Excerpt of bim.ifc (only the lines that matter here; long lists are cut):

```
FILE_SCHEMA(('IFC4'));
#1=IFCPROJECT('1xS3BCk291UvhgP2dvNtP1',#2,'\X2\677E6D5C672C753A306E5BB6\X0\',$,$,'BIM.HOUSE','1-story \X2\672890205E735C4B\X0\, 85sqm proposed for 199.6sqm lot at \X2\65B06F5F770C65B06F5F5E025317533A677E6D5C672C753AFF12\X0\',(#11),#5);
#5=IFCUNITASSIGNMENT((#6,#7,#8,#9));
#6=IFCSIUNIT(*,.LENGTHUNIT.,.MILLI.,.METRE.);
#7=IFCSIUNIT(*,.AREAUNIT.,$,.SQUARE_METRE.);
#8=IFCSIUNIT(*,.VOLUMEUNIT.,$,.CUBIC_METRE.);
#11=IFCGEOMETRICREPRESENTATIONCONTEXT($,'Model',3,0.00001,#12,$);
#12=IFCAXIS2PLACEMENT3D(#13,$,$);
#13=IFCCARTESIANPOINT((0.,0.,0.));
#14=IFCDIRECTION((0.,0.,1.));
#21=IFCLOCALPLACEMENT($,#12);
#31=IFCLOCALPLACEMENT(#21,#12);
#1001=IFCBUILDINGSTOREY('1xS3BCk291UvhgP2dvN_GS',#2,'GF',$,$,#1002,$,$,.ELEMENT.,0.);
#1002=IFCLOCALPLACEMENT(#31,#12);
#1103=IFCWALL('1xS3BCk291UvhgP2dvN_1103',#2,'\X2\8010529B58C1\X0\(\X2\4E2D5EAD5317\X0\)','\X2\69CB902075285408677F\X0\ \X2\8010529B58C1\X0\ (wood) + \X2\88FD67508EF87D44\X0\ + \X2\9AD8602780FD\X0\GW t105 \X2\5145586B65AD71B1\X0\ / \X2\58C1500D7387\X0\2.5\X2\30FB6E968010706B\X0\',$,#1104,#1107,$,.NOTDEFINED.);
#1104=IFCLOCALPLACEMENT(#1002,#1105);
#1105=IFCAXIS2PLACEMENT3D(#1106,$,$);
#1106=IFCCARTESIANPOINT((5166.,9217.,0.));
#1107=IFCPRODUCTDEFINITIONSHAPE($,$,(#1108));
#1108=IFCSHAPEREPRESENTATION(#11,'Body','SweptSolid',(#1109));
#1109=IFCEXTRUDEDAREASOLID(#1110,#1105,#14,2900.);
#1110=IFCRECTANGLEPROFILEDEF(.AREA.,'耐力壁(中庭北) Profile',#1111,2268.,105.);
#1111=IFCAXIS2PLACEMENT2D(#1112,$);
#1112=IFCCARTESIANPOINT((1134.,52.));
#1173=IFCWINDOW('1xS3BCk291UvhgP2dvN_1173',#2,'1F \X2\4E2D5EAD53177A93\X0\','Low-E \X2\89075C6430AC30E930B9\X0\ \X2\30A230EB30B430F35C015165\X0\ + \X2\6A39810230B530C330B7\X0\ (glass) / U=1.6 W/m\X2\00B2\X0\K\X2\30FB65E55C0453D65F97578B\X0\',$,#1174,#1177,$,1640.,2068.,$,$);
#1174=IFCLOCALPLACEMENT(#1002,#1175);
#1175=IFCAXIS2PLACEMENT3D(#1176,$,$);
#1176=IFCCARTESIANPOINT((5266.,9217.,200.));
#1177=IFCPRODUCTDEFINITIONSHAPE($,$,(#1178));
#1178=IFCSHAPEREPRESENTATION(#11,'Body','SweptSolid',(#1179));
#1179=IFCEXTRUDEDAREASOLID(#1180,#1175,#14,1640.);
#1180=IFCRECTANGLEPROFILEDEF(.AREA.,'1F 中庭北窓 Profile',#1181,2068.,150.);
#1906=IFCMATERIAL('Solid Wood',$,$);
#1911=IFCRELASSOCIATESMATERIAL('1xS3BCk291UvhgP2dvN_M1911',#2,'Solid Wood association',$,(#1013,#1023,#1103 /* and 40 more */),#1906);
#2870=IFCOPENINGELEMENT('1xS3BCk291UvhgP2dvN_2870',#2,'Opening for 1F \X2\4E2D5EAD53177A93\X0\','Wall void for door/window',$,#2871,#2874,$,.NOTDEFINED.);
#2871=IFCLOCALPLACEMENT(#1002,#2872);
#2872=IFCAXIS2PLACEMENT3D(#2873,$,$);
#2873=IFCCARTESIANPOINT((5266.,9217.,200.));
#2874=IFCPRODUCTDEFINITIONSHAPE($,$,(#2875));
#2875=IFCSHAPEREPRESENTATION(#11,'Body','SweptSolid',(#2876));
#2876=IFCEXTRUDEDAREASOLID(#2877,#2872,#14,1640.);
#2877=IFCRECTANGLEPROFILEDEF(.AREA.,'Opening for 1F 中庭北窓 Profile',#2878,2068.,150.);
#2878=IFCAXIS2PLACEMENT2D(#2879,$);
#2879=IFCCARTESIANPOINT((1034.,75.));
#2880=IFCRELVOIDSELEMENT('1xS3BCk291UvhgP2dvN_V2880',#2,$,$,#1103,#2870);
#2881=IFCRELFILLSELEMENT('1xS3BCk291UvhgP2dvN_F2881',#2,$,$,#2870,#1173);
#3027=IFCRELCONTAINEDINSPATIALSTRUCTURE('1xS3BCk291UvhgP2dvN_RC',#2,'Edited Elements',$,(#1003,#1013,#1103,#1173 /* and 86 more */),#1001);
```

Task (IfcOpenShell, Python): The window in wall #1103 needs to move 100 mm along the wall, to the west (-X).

```python
import ifcopenshell
import ifcopenshell.api.geometry
import ifcopenshell.util.placement

model = ifcopenshell.open("bim.ifc")

window = model.by_id(1173)
opening = window.FillsVoids[0].RelatingOpeningElement
wall = opening.VoidsElements[0].RelatingBuildingElement

wall_matrix = ifcopenshell.util.placement.get_local_placement(wall.ObjectPlacement)
shift = wall_matrix[:3, 0] * -100.0
before = ifcopenshell.util.placement.get_local_placement(window.ObjectPlacement)[:3, 3].copy()

# The window is not placed relative to its opening, so move both.
for product in (opening, window):
    matrix = ifcopenshell.util.placement.get_local_placement(product.ObjectPlacement)
    matrix[:3, 3] += shift
    ifcopenshell.api.geometry.edit_object_placement(model, product=product, matrix=matrix, is_si=False)

after = ifcopenshell.util.placement.get_local_placement(window.ObjectPlacement)[:3, 3]
print("window moved by", (after - before).round(3) + 0.0)

model.write("bim_rev.ifc")
```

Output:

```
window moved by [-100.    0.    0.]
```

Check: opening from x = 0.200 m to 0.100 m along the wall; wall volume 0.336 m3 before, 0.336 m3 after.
